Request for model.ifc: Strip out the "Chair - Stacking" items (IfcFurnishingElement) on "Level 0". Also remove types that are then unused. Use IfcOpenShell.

First a look at what the model holds.

```python
import ifcopenshell
import ifcopenshell.util.element

model = ifcopenshell.open("model.ifc")
print(model.schema)
storey = next(s for s in model.by_type("IfcBuildingStorey") if s.Name == "Level 0")
furniture = [e for e in ifcopenshell.util.element.get_decomposition(storey) if e.is_a("IfcFurnishingElement")]
seen = {}
for e in furniture:
    element_type = ifcopenshell.util.element.get_type(e)
    name = element_type.Name if element_type not in (None, e) else None
    seen[name] = seen.get(name, 0) + 1
for name, count in sorted(seen.items(), key=str):
    print(count, "x", name)
```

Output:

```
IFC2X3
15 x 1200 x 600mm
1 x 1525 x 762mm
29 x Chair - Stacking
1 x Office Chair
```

```python
import ifcopenshell
import ifcopenshell.api.root
import ifcopenshell.util.element

model = ifcopenshell.open("model.ifc")

storey = next(s for s in model.by_type("IfcBuildingStorey") if s.Name == "Level 0")
furniture = [e for e in ifcopenshell.util.element.get_decomposition(storey) if e.is_a("IfcFurnishingElement")]
targets = [e for e in furniture if (t := ifcopenshell.util.element.get_type(e)) not in (None, e) and t.Name == "Chair - Stacking"]
types = {ifcopenshell.util.element.get_type(e) for e in targets} - {None, *targets}

for e in targets:
    ifcopenshell.api.root.remove_product(model, product=e)
print(len(targets), "removed")

unused = [t for t in types if not ifcopenshell.util.element.get_types(t)]
for t in unused:
    ifcopenshell.api.root.remove_product(model, product=t)
print(len(unused), "unused types removed")

model.write("model_updated.ifc")
```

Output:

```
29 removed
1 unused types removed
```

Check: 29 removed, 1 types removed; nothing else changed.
